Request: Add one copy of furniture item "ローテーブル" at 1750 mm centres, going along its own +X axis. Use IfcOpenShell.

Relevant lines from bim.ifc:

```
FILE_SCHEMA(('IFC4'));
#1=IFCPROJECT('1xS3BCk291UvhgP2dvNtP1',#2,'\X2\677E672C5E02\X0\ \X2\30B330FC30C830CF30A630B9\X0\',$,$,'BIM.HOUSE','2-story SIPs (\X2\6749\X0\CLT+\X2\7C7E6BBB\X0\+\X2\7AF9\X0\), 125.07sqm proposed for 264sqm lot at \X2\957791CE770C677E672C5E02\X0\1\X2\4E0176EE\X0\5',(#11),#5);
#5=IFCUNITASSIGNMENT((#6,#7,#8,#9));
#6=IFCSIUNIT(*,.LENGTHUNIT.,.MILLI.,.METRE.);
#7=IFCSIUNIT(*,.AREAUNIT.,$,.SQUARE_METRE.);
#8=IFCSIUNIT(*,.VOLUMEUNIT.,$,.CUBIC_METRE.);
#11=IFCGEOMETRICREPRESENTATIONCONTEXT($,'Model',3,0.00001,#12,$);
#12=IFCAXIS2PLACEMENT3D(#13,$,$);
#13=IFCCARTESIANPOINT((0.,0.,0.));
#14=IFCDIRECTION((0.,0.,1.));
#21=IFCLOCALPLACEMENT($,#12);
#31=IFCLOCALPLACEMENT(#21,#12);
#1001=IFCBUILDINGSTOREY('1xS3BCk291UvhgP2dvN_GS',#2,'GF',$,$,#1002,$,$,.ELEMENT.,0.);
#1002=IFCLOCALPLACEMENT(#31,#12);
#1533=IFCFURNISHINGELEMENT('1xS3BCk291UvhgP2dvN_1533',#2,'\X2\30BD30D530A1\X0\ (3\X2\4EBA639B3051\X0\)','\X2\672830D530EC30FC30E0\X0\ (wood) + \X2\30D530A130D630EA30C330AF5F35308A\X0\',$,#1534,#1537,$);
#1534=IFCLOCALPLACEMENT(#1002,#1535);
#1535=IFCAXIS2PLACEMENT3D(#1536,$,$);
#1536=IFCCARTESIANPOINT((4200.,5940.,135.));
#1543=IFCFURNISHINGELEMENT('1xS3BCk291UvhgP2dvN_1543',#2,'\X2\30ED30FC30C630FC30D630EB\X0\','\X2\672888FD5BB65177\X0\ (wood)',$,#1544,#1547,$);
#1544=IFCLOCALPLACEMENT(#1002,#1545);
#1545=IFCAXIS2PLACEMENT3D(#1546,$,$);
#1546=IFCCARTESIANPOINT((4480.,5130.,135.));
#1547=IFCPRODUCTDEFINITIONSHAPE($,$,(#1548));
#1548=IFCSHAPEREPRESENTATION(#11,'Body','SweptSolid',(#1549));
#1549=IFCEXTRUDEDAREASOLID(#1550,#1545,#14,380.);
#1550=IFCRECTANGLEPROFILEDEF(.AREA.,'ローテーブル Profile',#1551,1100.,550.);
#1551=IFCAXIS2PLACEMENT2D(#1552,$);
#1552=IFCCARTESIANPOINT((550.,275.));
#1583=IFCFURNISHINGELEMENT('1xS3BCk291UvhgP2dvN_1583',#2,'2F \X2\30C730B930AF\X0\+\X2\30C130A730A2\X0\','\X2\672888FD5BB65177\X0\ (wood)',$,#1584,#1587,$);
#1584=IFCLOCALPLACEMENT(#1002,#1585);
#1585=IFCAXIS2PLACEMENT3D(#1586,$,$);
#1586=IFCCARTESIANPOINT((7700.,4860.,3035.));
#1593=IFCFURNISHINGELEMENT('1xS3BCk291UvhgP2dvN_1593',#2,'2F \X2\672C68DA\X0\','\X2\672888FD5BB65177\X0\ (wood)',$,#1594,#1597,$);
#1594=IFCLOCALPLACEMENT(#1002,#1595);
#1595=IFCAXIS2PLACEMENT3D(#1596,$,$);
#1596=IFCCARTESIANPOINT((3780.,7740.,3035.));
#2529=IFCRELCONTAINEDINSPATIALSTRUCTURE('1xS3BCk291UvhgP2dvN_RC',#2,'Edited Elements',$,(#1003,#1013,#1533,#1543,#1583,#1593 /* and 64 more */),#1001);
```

```python
import ifcopenshell
import ifcopenshell.api.geometry
import ifcopenshell.api.root
import ifcopenshell.util.element
import ifcopenshell.util.placement

model = ifcopenshell.open("bim.ifc")


def reuse_history(source, copy):
    """copy_class also copies each property set's owner history, people and application; keep the originals."""
    for rel in copy.IsDefinedBy:
        if rel.is_a("IfcRelDefinesByProperties") and (history := rel.RelatingPropertyDefinition.OwnerHistory):
            rel.RelatingPropertyDefinition.OwnerHistory = source.OwnerHistory
            ifcopenshell.util.element.remove_deep2(model, history)


source = model.by_guid("1xS3BCk291UvhgP2dvN_1543")
base = ifcopenshell.util.placement.get_local_placement(source.ObjectPlacement)
step = base[:3, 0] * 1750.0

for i in range(1, 2):
    copy = ifcopenshell.api.root.copy_class(model, product=source)
    copy.Representation = ifcopenshell.util.element.copy_deep(
        model, source.Representation, exclude=["IfcGeometricRepresentationContext", "IfcRepresentationMap"]
    )
    reuse_history(source, copy)
    matrix = base.copy()
    matrix[:3, 3] += i * step
    print("added at", matrix[:3, 3].round(3) + 0.0)
    ifcopenshell.api.geometry.edit_object_placement(model, product=copy, matrix=matrix, is_si=False)

model.write("bim-out.ifc")
```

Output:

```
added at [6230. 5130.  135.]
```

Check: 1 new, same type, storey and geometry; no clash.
